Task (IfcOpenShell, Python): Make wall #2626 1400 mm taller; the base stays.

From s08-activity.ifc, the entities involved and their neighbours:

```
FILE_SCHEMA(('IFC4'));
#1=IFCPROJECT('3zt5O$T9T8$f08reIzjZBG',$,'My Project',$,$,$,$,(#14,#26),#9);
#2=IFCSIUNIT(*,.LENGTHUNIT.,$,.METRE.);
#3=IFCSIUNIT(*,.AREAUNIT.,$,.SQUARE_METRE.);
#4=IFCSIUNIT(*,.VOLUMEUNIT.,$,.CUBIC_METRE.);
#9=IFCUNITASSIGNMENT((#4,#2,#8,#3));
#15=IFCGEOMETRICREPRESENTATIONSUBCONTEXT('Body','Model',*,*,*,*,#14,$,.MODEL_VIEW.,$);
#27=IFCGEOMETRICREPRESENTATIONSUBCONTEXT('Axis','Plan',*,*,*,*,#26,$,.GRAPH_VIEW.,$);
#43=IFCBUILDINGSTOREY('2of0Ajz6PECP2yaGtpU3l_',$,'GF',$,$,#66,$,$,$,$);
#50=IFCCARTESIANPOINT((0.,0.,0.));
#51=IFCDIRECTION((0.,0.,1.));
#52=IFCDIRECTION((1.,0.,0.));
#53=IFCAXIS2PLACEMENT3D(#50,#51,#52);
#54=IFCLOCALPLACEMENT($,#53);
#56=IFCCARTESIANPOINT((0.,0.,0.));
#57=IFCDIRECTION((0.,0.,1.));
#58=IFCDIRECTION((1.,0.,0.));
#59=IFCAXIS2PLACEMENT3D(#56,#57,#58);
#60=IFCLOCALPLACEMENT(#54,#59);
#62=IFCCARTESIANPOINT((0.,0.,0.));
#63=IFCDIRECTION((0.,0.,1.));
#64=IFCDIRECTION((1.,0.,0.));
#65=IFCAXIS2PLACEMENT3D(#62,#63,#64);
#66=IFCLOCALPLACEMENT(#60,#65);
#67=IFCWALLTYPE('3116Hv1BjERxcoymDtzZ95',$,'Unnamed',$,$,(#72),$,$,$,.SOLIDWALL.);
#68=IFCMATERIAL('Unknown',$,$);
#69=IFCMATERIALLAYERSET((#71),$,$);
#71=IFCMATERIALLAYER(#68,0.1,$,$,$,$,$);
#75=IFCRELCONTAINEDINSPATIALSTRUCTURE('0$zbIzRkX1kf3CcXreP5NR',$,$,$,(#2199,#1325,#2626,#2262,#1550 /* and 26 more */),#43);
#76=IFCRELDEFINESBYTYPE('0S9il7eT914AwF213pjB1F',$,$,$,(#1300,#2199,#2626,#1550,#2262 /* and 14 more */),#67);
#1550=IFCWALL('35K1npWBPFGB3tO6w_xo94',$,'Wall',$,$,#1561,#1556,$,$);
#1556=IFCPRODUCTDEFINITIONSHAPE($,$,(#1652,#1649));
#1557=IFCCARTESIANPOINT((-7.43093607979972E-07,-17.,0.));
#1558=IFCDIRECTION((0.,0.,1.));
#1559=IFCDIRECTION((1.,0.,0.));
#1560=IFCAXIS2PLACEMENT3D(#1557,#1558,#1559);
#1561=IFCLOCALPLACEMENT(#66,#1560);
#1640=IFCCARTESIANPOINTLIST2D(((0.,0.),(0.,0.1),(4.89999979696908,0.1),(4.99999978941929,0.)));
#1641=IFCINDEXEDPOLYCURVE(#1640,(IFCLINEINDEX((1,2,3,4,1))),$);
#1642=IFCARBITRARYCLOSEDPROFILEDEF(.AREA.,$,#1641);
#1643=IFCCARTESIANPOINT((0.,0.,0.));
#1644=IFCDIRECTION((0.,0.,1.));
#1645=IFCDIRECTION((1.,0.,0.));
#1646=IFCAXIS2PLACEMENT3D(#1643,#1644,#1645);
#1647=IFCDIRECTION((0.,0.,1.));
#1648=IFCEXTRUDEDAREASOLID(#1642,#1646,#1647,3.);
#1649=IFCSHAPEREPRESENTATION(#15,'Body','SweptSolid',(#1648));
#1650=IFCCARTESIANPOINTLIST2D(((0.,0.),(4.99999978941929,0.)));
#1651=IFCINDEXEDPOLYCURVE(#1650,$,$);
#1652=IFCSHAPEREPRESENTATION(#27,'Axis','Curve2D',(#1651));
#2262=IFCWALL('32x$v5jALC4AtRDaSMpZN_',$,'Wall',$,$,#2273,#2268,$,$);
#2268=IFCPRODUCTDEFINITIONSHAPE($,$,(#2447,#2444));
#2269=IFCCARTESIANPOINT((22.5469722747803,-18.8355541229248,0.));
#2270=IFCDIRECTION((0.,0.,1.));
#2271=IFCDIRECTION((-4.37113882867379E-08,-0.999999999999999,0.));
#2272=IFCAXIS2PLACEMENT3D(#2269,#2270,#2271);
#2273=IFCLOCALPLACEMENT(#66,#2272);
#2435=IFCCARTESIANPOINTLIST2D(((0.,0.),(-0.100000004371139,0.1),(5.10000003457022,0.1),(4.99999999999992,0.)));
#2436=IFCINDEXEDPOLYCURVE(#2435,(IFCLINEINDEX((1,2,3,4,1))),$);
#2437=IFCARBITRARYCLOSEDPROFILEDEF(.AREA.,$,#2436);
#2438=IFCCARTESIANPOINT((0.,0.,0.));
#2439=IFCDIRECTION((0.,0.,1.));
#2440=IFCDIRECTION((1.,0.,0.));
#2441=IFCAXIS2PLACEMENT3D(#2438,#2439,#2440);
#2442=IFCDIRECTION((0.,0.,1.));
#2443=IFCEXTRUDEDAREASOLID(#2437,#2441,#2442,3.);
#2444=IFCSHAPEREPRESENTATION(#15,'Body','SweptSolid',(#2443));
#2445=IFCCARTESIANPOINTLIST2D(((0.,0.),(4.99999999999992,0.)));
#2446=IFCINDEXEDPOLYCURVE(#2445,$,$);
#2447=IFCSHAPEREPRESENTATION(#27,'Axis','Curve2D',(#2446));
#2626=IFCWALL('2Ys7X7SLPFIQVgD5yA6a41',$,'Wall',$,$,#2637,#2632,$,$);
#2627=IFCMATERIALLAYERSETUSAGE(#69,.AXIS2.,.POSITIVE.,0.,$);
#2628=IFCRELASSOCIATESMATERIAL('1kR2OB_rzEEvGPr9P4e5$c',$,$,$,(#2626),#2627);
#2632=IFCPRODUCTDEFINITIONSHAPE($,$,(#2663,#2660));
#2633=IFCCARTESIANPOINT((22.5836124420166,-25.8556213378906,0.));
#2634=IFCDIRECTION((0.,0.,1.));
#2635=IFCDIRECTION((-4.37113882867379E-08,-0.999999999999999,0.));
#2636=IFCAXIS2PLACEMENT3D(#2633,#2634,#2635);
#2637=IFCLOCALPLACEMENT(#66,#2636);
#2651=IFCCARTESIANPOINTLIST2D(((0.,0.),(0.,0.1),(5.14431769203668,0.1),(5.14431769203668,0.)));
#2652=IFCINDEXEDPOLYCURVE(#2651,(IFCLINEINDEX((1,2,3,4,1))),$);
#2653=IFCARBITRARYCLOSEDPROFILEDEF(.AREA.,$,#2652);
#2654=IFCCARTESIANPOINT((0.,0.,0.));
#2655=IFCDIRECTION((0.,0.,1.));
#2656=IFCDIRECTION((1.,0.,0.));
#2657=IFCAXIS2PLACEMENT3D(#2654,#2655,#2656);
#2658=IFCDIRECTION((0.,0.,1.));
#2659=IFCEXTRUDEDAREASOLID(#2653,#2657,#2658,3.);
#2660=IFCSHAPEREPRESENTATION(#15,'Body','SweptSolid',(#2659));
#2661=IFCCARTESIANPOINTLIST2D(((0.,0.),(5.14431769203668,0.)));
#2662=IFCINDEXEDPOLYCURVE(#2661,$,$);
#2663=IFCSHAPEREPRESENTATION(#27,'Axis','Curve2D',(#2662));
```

```python
import ifcopenshell
import ifcopenshell.geom
import ifcopenshell.util.representation
import ifcopenshell.util.shape

model = ifcopenshell.open("s08-activity.ifc")
settings = ifcopenshell.geom.settings()


def volume(element):
    """Net volume in cubic metres, openings subtracted."""
    shape = ifcopenshell.geom.create_shape(settings, element)
    return ifcopenshell.util.shape.get_volume(shape.geometry)


wall = model.by_id(2626)
before = volume(wall)

body = ifcopenshell.util.representation.get_representation(wall, "Model", "Body")
solid = body.Items[0]
old_height = solid.Depth
solid.Depth += 1.4
after = volume(wall)

print(f"height {old_height:g} -> {solid.Depth:g}, volume {before:.3f} -> {after:.3f} m3")

model.write("s08-activity-out.ifc")
```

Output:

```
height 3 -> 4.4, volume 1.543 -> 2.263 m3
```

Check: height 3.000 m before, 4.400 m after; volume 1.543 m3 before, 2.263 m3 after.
